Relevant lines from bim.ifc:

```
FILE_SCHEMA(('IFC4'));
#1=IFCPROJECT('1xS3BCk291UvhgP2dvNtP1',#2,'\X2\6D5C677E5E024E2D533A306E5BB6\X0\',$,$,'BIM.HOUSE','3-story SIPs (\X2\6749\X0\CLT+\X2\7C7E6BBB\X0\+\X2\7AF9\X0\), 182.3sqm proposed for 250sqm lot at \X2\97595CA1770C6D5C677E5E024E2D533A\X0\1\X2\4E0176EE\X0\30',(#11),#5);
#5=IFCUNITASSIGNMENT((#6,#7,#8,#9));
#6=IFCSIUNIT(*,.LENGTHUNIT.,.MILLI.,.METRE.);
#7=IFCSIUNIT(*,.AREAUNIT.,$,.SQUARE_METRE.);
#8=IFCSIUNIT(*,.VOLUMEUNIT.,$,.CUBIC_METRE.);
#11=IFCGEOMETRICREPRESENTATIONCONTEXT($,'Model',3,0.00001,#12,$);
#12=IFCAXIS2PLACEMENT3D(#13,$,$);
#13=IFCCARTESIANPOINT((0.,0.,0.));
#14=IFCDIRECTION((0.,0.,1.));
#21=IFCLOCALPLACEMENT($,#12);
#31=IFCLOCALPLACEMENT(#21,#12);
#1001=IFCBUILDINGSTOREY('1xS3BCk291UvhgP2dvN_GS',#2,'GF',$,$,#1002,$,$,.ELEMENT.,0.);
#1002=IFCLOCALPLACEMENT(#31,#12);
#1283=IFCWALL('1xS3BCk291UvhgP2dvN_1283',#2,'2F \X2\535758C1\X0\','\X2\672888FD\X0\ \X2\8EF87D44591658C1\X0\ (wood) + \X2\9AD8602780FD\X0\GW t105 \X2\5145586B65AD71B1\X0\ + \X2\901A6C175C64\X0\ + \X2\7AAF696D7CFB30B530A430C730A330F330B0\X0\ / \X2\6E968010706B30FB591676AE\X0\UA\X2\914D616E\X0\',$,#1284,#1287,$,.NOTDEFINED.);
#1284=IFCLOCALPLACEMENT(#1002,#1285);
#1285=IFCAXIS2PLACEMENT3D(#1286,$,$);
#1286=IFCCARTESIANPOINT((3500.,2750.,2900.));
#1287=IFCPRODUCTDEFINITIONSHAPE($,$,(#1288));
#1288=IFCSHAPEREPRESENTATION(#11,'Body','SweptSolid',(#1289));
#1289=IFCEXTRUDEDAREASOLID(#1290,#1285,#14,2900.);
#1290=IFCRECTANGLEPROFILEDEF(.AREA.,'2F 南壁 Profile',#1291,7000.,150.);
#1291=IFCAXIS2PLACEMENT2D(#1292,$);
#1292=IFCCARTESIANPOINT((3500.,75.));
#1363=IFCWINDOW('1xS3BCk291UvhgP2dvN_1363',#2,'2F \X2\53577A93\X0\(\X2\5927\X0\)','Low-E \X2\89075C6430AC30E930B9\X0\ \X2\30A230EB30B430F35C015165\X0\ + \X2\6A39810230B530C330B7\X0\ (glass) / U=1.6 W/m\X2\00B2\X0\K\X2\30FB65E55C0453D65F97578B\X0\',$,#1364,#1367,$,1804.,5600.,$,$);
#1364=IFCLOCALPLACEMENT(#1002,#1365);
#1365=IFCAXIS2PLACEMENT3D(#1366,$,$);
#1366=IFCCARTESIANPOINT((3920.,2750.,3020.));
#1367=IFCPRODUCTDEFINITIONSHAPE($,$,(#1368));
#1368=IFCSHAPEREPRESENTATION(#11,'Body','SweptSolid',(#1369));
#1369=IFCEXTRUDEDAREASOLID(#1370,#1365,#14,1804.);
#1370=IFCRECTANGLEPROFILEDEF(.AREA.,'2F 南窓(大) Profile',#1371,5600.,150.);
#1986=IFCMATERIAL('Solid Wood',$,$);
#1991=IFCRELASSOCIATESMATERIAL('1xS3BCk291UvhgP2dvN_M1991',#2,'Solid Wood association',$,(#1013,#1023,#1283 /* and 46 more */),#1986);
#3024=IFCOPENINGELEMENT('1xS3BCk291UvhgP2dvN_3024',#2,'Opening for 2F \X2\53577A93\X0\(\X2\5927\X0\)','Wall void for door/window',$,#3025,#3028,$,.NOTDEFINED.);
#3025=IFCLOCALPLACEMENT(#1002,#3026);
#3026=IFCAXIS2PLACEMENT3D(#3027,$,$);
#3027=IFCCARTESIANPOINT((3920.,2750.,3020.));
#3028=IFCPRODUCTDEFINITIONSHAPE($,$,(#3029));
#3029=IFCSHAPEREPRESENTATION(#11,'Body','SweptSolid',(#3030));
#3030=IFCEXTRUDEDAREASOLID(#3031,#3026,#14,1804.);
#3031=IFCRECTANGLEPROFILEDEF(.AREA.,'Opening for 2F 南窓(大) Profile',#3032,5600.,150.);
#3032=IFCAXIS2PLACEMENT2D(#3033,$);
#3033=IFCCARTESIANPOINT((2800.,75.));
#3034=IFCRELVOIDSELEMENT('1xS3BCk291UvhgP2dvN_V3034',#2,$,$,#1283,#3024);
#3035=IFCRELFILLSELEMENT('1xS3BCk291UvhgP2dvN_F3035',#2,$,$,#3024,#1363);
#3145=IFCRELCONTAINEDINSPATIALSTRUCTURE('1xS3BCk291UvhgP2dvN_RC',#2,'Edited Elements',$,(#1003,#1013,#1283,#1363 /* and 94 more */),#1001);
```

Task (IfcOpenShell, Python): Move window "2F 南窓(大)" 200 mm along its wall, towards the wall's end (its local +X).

```python
import ifcopenshell
import ifcopenshell.api.geometry
import ifcopenshell.util.placement
import ifcopenshell.util.unit

model = ifcopenshell.open("bim.ifc")
unit_scale = ifcopenshell.util.unit.calculate_unit_scale(model)

window = model.by_id(1363)
opening = window.FillsVoids[0].RelatingOpeningElement
wall = opening.VoidsElements[0].RelatingBuildingElement

wall_matrix = ifcopenshell.util.placement.get_local_placement(wall.ObjectPlacement)
shift = wall_matrix[:3, 0] * 0.2 / unit_scale
before = ifcopenshell.util.placement.get_local_placement(window.ObjectPlacement)[:3, 3].copy()

# The window is not placed relative to its opening, so move both.
for product in (opening, window):
    matrix = ifcopenshell.util.placement.get_local_placement(product.ObjectPlacement)
    matrix[:3, 3] += shift
    ifcopenshell.api.geometry.edit_object_placement(model, product=product, matrix=matrix, is_si=False)

after = ifcopenshell.util.placement.get_local_placement(window.ObjectPlacement)[:3, 3]
print("window moved by", (after - before).round(3) + 0.0)

model.write("bim-out.ifc")
```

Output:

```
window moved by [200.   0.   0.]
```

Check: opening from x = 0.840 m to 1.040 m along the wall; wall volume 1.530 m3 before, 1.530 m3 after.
